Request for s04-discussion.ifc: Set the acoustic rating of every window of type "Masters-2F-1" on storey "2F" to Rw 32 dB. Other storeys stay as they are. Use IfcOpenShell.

First a look at what the model holds.

```python
import ifcopenshell
import ifcopenshell.util.element

model = ifcopenshell.open("s04-discussion.ifc")
print(model.schema)
storey = next(s for s in model.by_type("IfcBuildingStorey") if s.Name == "2F")
windows = [e for e in ifcopenshell.util.element.get_decomposition(storey) if e.is_a("IfcWindow")]
seen = {}
for e in windows:
    element_type = ifcopenshell.util.element.get_type(e)
    key = (element_type.Name if element_type != e and element_type else None, ifcopenshell.util.element.get_pset(e, "Pset_WindowCommon", "AcousticRating"))
    seen[key] = seen.get(key, 0) + 1
for (name, value), count in sorted(seen.items(), key=str):
    print(count, "x", name, "|", value)
```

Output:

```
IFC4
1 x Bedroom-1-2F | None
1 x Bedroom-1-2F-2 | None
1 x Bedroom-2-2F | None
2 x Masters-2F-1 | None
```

```python
import ifcopenshell
import ifcopenshell.api.pset
import ifcopenshell.util.element

model = ifcopenshell.open("s04-discussion.ifc")

storey = next(s for s in model.by_type("IfcBuildingStorey") if s.Name == "2F")
windows = [e for e in ifcopenshell.util.element.get_decomposition(storey) if e.is_a("IfcWindow")]

count = 0
for e in windows:
    element_type = ifcopenshell.util.element.get_type(e)
    if element_type in (None, e) or element_type.Name != "Masters-2F-1":
        continue
    # add_pset returns the element's existing set when there is one.
    pset = ifcopenshell.api.pset.add_pset(model, product=e, name="Pset_WindowCommon")
    ifcopenshell.api.pset.edit_pset(model, pset=pset, properties={"AcousticRating": "Rw 32 dB"})
    count += 1

print(count, "windows updated")

model.write("s04-discussion_updated.ifc")
```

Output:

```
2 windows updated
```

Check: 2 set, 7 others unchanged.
